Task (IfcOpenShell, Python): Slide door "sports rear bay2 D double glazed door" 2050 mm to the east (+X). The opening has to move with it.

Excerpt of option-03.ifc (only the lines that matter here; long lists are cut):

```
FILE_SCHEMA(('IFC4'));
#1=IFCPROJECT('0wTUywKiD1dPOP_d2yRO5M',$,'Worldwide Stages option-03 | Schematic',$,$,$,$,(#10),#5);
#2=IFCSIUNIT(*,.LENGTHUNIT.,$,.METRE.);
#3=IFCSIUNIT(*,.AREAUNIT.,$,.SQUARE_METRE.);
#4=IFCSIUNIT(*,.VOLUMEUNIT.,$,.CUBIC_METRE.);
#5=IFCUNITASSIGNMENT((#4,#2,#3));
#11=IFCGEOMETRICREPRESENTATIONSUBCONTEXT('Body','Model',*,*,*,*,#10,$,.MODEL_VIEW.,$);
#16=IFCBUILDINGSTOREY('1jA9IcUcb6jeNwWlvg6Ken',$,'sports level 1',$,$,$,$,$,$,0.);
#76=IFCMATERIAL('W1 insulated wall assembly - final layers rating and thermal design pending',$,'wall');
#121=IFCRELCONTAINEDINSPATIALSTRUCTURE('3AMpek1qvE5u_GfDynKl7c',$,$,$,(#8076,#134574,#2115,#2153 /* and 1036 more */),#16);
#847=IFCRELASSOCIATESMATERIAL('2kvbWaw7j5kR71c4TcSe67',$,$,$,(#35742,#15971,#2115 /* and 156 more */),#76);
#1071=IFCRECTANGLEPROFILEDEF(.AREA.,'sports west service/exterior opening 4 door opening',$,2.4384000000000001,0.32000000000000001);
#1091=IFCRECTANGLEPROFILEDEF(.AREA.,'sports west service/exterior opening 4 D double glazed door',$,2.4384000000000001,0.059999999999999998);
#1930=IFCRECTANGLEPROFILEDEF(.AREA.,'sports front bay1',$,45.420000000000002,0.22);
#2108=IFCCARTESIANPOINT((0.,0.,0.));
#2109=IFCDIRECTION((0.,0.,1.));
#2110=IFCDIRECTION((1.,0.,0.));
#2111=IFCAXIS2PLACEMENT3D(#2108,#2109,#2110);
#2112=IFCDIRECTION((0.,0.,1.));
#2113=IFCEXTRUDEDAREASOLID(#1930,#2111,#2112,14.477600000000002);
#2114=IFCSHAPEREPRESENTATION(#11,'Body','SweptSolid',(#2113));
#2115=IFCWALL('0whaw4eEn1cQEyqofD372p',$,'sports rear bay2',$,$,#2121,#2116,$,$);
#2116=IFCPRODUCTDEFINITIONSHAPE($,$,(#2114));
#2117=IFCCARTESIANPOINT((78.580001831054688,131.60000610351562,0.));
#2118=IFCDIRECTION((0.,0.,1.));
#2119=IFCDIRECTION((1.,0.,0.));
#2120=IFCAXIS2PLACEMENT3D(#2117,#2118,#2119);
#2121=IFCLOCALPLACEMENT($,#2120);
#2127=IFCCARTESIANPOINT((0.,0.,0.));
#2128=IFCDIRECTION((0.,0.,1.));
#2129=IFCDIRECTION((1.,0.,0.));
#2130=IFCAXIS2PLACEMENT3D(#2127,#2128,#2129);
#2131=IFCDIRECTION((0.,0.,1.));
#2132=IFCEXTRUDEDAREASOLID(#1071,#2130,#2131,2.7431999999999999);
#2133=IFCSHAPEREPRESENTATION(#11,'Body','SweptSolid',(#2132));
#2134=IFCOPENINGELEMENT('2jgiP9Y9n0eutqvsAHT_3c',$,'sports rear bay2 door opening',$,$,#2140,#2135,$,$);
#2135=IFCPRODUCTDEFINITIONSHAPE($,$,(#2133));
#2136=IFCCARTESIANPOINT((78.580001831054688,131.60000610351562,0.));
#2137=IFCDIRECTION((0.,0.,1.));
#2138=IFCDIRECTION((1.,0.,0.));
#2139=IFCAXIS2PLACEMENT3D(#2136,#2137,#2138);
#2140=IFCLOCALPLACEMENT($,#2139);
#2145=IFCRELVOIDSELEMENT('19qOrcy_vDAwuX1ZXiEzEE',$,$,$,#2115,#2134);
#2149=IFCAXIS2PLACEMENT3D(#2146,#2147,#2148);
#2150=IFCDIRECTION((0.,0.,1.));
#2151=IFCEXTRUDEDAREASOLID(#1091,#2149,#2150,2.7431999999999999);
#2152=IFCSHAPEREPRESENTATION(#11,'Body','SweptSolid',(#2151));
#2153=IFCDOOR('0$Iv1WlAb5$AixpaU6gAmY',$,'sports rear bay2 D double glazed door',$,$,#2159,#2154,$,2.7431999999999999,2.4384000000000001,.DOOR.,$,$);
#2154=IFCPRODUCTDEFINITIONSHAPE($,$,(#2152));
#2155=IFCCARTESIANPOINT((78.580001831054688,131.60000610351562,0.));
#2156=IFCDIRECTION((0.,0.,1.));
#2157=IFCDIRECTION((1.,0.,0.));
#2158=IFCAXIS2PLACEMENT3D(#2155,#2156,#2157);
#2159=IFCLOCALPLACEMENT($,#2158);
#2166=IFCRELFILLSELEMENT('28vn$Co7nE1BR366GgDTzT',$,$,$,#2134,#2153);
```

```python
import ifcopenshell
import ifcopenshell.api.geometry
import ifcopenshell.util.placement
import ifcopenshell.util.unit

model = ifcopenshell.open("option-03.ifc")
unit_scale = ifcopenshell.util.unit.calculate_unit_scale(model)

door = model.by_id(2153)
opening = door.FillsVoids[0].RelatingOpeningElement
wall = opening.VoidsElements[0].RelatingBuildingElement

wall_matrix = ifcopenshell.util.placement.get_local_placement(wall.ObjectPlacement)
shift = wall_matrix[:3, 0] * 2.05 / unit_scale
before = ifcopenshell.util.placement.get_local_placement(door.ObjectPlacement)[:3, 3].copy()

# The door is not placed relative to its opening, so move both.
for product in (opening, door):
    matrix = ifcopenshell.util.placement.get_local_placement(product.ObjectPlacement)
    matrix[:3, 3] += shift
    ifcopenshell.api.geometry.edit_object_placement(model, product=product, matrix=matrix, is_si=False)

after = ifcopenshell.util.placement.get_local_placement(door.ObjectPlacement)[:3, 3]
print("door moved by", (after - before).round(3) + 0.0)

model.write("option-03-out.ifc")
```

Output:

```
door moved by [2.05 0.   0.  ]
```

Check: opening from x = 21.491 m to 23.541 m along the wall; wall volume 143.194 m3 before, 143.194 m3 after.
